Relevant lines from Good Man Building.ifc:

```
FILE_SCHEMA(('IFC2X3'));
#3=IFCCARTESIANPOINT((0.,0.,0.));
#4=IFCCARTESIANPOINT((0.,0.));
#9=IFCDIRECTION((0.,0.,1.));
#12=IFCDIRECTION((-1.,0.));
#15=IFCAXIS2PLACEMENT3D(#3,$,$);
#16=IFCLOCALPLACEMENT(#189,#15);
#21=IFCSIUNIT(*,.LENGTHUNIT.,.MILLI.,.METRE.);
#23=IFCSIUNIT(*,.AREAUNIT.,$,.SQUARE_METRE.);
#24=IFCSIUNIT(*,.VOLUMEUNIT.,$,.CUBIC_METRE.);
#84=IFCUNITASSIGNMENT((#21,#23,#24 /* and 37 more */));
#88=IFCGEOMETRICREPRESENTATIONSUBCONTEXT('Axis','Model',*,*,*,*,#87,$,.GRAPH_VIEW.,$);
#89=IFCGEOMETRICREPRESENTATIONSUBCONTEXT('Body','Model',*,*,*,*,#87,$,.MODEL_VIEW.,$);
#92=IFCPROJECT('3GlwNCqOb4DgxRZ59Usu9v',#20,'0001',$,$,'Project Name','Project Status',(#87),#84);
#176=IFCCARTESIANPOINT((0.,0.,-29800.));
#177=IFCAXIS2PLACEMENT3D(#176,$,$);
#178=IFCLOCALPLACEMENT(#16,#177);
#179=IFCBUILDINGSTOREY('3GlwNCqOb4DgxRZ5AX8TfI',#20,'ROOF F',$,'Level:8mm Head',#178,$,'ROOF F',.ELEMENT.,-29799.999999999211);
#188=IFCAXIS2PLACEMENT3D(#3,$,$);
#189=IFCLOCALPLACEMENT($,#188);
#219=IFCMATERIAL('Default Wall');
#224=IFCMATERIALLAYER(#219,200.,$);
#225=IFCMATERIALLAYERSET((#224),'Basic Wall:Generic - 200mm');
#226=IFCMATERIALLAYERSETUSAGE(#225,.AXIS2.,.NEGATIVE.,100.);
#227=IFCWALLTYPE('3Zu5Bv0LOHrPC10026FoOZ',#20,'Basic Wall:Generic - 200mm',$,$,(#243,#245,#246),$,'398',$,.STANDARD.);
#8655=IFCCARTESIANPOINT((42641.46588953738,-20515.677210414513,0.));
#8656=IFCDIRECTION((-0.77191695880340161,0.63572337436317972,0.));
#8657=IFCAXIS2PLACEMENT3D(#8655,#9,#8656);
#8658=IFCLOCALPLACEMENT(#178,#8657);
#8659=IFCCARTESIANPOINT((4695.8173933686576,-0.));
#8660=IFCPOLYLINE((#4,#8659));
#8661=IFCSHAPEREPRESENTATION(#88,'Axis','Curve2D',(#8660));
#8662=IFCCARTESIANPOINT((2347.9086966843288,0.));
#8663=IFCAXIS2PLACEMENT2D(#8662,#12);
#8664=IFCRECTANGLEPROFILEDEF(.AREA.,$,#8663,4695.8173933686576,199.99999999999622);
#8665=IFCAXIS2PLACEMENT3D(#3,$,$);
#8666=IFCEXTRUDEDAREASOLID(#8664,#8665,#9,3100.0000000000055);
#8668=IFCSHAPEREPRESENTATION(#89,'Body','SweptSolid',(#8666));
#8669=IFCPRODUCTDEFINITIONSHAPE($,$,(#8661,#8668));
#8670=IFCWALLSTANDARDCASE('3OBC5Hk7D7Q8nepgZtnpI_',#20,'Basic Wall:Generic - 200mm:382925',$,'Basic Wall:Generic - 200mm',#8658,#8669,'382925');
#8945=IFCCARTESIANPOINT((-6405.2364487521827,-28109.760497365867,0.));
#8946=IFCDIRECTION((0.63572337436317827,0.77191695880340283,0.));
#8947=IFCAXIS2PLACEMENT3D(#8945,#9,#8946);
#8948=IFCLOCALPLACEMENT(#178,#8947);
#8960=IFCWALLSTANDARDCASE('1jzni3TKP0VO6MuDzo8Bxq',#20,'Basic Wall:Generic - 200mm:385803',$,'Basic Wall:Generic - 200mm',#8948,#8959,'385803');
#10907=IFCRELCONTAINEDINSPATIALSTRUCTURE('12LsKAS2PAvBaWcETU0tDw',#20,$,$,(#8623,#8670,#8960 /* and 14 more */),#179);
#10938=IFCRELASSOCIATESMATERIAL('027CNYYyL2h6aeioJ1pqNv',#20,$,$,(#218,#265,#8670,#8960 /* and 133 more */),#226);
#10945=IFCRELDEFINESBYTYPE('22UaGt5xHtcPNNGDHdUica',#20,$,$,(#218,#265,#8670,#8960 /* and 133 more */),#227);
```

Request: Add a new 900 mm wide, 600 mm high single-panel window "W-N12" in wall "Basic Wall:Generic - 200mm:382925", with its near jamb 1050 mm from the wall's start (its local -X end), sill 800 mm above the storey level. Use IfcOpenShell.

```python
import numpy as np
import ifcopenshell
import ifcopenshell.api.feature
import ifcopenshell.api.geometry
import ifcopenshell.api.root
import ifcopenshell.api.spatial
import ifcopenshell.api.type
import ifcopenshell.geom
import ifcopenshell.util.element
import ifcopenshell.util.placement
import ifcopenshell.util.representation
import ifcopenshell.util.shape
import ifcopenshell.util.unit

model = ifcopenshell.open("Good Man Building.ifc")
unit_scale = ifcopenshell.util.unit.calculate_unit_scale(model)
settings = ifcopenshell.geom.settings()


def volume(element):
    """Net volume in cubic metres, openings subtracted."""
    shape = ifcopenshell.geom.create_shape(settings, element)
    return ifcopenshell.util.shape.get_volume(shape.geometry)


wall = model.by_guid("3OBC5Hk7D7Q8nepgZtnpI_")
storey = ifcopenshell.util.element.get_container(wall, ifc_class="IfcBuildingStorey")
context = ifcopenshell.util.representation.get_context(model, "Model", "Body", "MODEL_VIEW")
before = volume(wall)

width, height, from_end, sill = 0.9, 0.6, 1.05, 0.8  # metres

# The wall runs along its own X axis, and the end named is its -X end.
wall_shape = ifcopenshell.geom.create_shape(settings, wall)
x, y, z = ifcopenshell.util.shape.get_vertices(wall_shape.geometry).T
start = x.min() + from_end
face, thickness = float(y.min()), float(y.max() - y.min())
wall_matrix = ifcopenshell.util.placement.get_local_placement(wall.ObjectPlacement)
level = ifcopenshell.util.placement.get_local_placement(storey.ObjectPlacement)[2, 3]


def in_wall(x, y):
    """Placement at x, y metres in the wall's axes, at sill height."""
    matrix = wall_matrix.copy()
    matrix[:, 3] = wall_matrix @ np.array([x / unit_scale, y / unit_scale, 0.0, 1.0])
    matrix[2, 3] = level + sill / unit_scale
    return matrix


# Opening: a box that overshoots both wall faces by 50 mm.
opening = ifcopenshell.api.root.create_entity(model, ifc_class="IfcOpeningElement")
box = ifcopenshell.api.geometry.add_wall_representation(
    model, context=context, length=width, height=height, thickness=thickness + 0.1
)
ifcopenshell.api.geometry.assign_representation(model, product=opening, representation=box)
ifcopenshell.api.geometry.edit_object_placement(model, product=opening, matrix=in_wall(start, face - 0.05), is_si=False)
ifcopenshell.api.feature.add_feature(model, feature=opening, element=wall)

window = ifcopenshell.api.root.create_entity(model, ifc_class="IfcWindow", name="W-N12")
window.OverallWidth, window.OverallHeight = width / unit_scale, height / unit_scale
body = ifcopenshell.api.geometry.add_window_representation(
    model,
    context=context,
    overall_width=window.OverallWidth,
    overall_height=window.OverallHeight,
    partition_type="SINGLE_PANEL",
)
ifcopenshell.api.geometry.assign_representation(model, product=window, representation=body)
ifcopenshell.api.spatial.assign_container(model, products=[window], relating_structure=storey)
fills = ifcopenshell.api.feature.add_filling(model, opening=opening, element=window)
fills.OwnerHistory = window.OwnerHistory  # required in IFC2X3

# IFC2X3 keeps the operation on the window style.
style = ifcopenshell.api.root.create_entity(model, ifc_class="IfcWindowStyle", name="W-N12")
style.OperationType, style.ConstructionType = "SINGLE_PANEL", "NOTDEFINED"
style.ParameterTakesPrecedence = style.Sizeable = False
ifcopenshell.api.type.assign_type(model, related_objects=[window], relating_type=style)

# Centre the window in the wall's thickness.
ifcopenshell.api.geometry.edit_object_placement(model, product=window, matrix=in_wall(start, face), is_si=False)
window_shape = ifcopenshell.geom.create_shape(settings, window)
depth = ifcopenshell.util.shape.get_vertices(window_shape.geometry)[:, 1]
offset = face + thickness / 2 - (depth.min() + depth.max()) / 2
ifcopenshell.api.geometry.edit_object_placement(model, product=window, matrix=in_wall(start, offset), is_si=False)

after = volume(wall)

print(f"wall volume {before:.3f} -> {after:.3f} m3")

model.write("Good Man Building_rev.ifc")
```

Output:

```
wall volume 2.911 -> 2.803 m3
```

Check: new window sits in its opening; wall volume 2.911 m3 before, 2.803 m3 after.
